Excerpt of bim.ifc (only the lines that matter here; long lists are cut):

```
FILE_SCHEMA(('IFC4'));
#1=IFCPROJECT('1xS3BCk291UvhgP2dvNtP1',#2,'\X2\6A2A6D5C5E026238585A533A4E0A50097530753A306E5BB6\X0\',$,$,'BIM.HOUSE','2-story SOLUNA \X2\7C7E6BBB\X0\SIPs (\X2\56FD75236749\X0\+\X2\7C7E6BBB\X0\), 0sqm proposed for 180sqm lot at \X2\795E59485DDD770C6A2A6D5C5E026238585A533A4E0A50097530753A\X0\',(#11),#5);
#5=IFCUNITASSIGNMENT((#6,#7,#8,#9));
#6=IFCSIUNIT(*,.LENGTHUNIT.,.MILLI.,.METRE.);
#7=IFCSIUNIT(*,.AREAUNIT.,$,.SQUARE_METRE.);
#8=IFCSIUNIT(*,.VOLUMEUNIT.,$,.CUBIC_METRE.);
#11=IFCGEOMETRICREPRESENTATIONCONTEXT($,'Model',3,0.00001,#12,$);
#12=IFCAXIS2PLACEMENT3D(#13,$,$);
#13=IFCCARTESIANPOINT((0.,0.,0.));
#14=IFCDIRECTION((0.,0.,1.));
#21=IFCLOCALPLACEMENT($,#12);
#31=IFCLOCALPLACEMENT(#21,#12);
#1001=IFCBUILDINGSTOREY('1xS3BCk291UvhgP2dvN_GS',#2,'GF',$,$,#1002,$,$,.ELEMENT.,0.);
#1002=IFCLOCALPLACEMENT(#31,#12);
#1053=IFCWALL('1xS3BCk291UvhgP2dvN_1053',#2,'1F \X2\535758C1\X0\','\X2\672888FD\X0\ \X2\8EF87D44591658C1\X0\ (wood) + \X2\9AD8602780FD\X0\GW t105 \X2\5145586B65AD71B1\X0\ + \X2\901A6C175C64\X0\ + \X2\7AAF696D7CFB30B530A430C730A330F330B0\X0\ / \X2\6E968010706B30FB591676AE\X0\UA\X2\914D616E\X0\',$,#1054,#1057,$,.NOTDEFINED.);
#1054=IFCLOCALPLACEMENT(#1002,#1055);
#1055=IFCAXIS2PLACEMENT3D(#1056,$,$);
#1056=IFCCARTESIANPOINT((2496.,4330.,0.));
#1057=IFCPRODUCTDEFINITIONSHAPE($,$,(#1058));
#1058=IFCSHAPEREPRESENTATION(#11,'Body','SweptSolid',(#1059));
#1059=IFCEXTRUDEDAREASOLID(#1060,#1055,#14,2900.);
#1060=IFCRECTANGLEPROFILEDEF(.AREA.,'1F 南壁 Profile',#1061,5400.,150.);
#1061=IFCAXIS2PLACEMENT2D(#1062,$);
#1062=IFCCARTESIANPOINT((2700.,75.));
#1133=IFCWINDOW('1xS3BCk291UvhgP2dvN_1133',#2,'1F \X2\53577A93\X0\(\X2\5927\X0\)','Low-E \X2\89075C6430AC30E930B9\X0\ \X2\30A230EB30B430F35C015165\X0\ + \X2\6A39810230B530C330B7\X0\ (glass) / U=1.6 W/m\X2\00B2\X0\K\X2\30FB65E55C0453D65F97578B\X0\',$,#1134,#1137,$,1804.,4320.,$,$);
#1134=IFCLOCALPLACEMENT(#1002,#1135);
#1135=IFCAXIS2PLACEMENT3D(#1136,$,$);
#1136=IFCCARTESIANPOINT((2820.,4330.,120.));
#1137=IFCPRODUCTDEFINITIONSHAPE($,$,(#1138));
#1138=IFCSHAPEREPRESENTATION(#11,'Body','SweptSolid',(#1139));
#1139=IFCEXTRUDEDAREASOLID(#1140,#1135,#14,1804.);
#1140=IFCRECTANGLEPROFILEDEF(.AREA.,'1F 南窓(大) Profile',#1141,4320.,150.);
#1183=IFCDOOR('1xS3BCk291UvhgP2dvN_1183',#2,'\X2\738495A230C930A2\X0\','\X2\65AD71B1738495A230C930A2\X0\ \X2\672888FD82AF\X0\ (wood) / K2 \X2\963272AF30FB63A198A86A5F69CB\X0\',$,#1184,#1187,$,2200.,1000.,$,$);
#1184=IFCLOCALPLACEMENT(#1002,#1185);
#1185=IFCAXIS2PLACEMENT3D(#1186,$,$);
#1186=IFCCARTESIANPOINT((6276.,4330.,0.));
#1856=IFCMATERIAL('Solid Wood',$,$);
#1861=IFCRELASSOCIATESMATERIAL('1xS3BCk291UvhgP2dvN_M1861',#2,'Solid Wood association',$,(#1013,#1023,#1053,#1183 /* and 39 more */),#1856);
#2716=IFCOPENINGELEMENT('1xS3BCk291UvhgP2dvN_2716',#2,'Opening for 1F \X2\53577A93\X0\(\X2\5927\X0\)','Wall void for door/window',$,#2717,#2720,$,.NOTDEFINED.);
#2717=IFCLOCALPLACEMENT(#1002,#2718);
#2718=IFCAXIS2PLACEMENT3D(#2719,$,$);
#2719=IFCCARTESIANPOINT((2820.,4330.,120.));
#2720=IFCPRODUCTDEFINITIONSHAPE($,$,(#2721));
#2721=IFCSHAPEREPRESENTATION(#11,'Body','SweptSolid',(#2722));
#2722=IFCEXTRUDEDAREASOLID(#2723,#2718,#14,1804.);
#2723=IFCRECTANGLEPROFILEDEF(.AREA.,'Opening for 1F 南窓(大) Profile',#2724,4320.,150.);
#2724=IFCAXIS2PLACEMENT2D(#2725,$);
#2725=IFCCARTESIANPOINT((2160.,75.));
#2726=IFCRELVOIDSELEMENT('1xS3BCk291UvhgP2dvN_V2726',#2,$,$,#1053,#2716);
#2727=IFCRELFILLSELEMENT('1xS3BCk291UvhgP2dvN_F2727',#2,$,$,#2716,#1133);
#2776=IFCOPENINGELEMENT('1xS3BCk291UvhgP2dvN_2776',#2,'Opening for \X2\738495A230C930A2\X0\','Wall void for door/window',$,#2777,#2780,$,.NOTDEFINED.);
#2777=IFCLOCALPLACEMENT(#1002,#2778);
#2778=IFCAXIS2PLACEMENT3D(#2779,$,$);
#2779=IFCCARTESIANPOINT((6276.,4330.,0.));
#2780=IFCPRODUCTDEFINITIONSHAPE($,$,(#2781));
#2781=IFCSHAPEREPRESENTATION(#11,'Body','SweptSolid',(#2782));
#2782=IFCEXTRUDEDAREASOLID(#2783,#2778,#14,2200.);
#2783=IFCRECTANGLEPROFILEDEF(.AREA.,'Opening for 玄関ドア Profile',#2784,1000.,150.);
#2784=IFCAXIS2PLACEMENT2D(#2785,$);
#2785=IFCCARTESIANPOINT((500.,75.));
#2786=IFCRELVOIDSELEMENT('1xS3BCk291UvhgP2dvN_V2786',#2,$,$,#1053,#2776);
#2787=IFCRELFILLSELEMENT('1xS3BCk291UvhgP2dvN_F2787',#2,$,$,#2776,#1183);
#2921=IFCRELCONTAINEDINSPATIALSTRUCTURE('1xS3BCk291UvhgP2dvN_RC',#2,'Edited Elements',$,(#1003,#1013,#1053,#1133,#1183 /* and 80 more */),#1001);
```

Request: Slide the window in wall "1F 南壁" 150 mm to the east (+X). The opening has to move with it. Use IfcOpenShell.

```python
import ifcopenshell
import ifcopenshell.api.geometry
import ifcopenshell.util.placement
import ifcopenshell.util.unit

model = ifcopenshell.open("bim.ifc")
unit_scale = ifcopenshell.util.unit.calculate_unit_scale(model)

window = model.by_guid("1xS3BCk291UvhgP2dvN_1133")
opening = window.FillsVoids[0].RelatingOpeningElement
wall = opening.VoidsElements[0].RelatingBuildingElement

wall_matrix = ifcopenshell.util.placement.get_local_placement(wall.ObjectPlacement)
shift = wall_matrix[:3, 0] * 0.15 / unit_scale
before = ifcopenshell.util.placement.get_local_placement(window.ObjectPlacement)[:3, 3].copy()

# The window is not placed relative to its opening, so move both.
for product in (opening, window):
    matrix = ifcopenshell.util.placement.get_local_placement(product.ObjectPlacement)
    matrix[:3, 3] += shift
    ifcopenshell.api.geometry.edit_object_placement(model, product=product, matrix=matrix, is_si=False)

after = ifcopenshell.util.placement.get_local_placement(window.ObjectPlacement)[:3, 3]
print("window moved by", (after - before).round(3) + 0.0)

model.write("bim_v2.ifc")
```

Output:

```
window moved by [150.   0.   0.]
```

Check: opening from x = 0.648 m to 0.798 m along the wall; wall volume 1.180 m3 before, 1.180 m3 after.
